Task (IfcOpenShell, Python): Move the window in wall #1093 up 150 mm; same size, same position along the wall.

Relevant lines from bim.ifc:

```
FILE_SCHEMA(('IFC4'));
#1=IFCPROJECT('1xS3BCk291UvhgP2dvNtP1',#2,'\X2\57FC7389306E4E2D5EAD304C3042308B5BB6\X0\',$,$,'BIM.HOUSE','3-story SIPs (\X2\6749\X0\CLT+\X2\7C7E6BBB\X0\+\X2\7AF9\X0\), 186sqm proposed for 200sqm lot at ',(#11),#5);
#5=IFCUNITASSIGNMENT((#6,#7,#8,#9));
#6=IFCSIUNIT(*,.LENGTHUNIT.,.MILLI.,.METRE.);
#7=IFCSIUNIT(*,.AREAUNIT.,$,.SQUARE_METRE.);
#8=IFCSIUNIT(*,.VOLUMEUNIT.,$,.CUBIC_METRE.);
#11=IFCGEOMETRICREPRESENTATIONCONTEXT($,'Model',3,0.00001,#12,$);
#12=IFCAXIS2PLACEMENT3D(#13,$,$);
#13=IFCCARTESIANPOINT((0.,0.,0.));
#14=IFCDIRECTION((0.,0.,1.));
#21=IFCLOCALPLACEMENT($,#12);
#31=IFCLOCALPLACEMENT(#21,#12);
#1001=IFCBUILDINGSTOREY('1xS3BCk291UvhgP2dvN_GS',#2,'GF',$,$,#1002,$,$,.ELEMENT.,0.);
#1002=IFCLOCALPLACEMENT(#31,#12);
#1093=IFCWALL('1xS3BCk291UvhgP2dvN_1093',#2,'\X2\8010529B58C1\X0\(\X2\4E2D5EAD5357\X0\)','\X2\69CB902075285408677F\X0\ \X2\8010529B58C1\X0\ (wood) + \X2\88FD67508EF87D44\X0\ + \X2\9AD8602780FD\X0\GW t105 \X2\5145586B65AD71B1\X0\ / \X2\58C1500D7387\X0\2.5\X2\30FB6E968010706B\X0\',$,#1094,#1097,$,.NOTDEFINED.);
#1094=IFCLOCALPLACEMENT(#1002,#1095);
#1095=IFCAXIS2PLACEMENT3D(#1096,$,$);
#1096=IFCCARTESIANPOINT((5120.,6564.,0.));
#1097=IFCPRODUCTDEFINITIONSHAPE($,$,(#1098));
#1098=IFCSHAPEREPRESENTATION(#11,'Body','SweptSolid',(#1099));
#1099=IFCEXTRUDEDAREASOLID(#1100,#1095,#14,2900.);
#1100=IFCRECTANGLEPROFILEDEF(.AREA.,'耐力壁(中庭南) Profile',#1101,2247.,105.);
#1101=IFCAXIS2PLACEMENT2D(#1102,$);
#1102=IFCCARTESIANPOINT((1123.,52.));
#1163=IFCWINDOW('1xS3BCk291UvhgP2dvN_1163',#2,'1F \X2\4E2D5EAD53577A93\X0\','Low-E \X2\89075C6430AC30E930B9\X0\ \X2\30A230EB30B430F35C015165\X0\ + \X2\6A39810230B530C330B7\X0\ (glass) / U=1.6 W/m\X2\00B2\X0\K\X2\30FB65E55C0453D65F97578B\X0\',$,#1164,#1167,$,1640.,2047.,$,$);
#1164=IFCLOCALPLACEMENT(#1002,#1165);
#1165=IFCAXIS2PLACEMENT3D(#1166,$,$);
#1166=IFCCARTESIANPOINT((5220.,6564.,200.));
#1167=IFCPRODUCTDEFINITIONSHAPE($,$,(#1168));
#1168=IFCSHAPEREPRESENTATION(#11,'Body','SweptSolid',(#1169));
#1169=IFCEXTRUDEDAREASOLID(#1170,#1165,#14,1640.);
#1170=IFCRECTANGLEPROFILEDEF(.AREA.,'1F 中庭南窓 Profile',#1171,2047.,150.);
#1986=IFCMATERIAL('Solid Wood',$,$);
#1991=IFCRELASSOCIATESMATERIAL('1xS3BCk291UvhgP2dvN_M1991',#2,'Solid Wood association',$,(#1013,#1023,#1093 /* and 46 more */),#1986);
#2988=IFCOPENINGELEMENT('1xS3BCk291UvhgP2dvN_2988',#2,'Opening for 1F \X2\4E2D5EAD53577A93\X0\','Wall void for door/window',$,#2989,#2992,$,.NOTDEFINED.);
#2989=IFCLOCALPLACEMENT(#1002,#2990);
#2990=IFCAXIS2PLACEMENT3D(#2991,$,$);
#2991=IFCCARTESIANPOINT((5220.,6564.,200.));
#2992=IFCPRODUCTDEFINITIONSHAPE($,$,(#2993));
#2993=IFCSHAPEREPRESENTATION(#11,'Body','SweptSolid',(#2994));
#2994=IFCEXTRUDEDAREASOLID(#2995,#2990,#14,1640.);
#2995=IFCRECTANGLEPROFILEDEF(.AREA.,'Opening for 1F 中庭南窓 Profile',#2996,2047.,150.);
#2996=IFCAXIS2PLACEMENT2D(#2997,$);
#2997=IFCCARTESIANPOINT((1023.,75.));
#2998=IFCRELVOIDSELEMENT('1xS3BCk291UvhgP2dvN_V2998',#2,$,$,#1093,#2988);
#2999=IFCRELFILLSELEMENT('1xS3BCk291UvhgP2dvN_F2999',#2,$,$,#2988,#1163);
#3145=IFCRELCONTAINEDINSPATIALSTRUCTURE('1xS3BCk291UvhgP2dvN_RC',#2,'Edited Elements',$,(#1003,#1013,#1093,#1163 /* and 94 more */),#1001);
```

```python
import numpy as np
import ifcopenshell
import ifcopenshell.api.geometry
import ifcopenshell.util.placement
import ifcopenshell.util.unit

model = ifcopenshell.open("bim.ifc")
unit_scale = ifcopenshell.util.unit.calculate_unit_scale(model)

window = model.by_id(1163)
opening = window.FillsVoids[0].RelatingOpeningElement
dz = 0.15 / unit_scale

shift = np.array([0.0, 0.0, dz])
# The window is not placed relative to its opening, so move both.
for product in (opening, window):
    matrix = ifcopenshell.util.placement.get_local_placement(product.ObjectPlacement)
    matrix[:3, 3] += shift
    ifcopenshell.api.geometry.edit_object_placement(model, product=product, matrix=matrix, is_si=False)

print(f"moved by {dz * unit_scale:+.3f} m")

model.write("bim_v2.ifc")
```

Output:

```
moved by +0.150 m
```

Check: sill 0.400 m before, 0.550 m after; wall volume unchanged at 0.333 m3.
